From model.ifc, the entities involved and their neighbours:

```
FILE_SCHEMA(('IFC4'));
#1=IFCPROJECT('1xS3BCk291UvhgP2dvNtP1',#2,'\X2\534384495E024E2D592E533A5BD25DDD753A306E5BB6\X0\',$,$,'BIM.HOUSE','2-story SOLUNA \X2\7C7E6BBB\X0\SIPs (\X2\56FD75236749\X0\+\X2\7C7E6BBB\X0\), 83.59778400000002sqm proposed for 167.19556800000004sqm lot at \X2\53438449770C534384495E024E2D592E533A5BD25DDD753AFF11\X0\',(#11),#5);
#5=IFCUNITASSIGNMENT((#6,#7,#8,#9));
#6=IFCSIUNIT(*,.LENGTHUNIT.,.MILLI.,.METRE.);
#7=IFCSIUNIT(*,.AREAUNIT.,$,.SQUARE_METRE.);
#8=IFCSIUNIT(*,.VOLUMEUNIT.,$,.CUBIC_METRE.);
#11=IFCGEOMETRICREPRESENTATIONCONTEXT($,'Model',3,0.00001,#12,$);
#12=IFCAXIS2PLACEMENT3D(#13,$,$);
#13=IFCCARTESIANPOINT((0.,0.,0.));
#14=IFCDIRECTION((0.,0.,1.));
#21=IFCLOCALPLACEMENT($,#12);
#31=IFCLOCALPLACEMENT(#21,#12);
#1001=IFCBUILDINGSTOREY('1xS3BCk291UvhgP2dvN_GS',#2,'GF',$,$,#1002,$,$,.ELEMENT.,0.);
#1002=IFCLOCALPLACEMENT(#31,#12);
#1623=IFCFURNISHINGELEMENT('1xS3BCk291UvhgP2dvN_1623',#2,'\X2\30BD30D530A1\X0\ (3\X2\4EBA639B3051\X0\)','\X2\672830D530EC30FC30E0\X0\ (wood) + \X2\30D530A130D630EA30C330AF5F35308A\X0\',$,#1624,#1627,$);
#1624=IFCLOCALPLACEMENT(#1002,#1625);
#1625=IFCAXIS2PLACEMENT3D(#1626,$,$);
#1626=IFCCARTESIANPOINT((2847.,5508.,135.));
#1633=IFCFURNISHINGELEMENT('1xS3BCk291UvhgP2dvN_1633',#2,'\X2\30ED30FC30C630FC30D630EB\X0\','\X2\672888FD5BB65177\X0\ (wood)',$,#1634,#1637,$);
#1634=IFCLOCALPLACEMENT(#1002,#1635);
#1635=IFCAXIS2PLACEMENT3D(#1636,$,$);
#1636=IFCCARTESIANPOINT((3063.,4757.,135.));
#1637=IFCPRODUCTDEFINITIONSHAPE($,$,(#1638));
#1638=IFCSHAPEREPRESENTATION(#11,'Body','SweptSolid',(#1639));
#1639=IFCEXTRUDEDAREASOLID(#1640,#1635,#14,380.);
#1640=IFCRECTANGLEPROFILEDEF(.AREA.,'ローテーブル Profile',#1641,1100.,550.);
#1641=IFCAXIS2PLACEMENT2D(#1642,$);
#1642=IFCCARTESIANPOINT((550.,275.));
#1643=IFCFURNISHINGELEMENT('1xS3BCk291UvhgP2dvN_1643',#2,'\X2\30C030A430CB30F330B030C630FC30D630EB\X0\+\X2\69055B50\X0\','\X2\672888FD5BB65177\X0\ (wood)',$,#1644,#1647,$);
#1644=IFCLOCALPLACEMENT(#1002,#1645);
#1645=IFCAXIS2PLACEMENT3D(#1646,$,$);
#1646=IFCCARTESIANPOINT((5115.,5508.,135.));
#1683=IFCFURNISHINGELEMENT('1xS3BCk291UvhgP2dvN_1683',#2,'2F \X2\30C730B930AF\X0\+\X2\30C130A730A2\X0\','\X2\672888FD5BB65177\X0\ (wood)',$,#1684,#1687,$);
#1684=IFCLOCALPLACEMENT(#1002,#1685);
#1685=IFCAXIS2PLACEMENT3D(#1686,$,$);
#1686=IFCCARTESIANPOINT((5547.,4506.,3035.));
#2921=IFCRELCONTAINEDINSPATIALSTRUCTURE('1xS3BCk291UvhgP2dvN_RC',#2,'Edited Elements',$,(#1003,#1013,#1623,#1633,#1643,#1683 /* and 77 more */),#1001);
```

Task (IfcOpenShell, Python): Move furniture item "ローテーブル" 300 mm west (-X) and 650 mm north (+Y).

```python
import ifcopenshell
import ifcopenshell.api.geometry
import ifcopenshell.util.placement
import ifcopenshell.util.unit

model = ifcopenshell.open("model.ifc")
unit_scale = ifcopenshell.util.unit.calculate_unit_scale(model)

item = model.by_guid("1xS3BCk291UvhgP2dvN_1633")
matrix = ifcopenshell.util.placement.get_local_placement(item.ObjectPlacement)
matrix[0, 3] -= 0.3 / unit_scale
matrix[1, 3] += 0.65 / unit_scale
ifcopenshell.api.geometry.edit_object_placement(model, product=item, matrix=matrix, is_si=False)

print(ifcopenshell.util.placement.get_local_placement(item.ObjectPlacement).round(3) + 0.0)

model.write("model_edited.ifc")
```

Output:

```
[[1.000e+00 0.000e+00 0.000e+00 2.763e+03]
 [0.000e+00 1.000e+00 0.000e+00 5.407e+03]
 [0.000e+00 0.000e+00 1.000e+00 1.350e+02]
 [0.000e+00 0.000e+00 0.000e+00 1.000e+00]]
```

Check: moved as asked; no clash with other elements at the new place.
